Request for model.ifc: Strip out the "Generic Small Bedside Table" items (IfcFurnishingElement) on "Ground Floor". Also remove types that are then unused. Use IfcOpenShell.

First a look at what the model holds.

```python
import ifcopenshell
import ifcopenshell.util.element

model = ifcopenshell.open("model.ifc")
print(model.schema)
storey = next(s for s in model.by_type("IfcBuildingStorey") if s.Name == "Ground Floor")
furniture = [e for e in ifcopenshell.util.element.get_decomposition(storey) if e.is_a("IfcFurnishingElement")]
seen = {}
for e in furniture:
    element_type = ifcopenshell.util.element.get_type(e)
    name = element_type.Name if element_type not in (None, e) else None
    seen[name] = seen.get(name, 0) + 1
for name, count in sorted(seen.items(), key=str):
    print(count, "x", name)
```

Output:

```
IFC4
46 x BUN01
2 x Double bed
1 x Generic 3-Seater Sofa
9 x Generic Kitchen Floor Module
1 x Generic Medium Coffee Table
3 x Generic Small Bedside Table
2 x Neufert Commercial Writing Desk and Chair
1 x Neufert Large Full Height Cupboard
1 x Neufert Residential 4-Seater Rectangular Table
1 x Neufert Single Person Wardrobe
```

```python
import ifcopenshell
import ifcopenshell.api.root
import ifcopenshell.util.element

model = ifcopenshell.open("model.ifc")

storey = next(s for s in model.by_type("IfcBuildingStorey") if s.Name == "Ground Floor")
furniture = [e for e in ifcopenshell.util.element.get_decomposition(storey) if e.is_a("IfcFurnishingElement")]
targets = [e for e in furniture if (t := ifcopenshell.util.element.get_type(e)) not in (None, e) and t.Name == "Generic Small Bedside Table"]
types = {ifcopenshell.util.element.get_type(e) for e in targets} - {None, *targets}

for e in targets:
    ifcopenshell.api.root.remove_product(model, product=e)
print(len(targets), "removed")

unused = [t for t in types if not ifcopenshell.util.element.get_types(t)]
for t in unused:
    ifcopenshell.api.root.remove_product(model, product=t)
print(len(unused), "unused types removed")

model.write("model-out.ifc")
```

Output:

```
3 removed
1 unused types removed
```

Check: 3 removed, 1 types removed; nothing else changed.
